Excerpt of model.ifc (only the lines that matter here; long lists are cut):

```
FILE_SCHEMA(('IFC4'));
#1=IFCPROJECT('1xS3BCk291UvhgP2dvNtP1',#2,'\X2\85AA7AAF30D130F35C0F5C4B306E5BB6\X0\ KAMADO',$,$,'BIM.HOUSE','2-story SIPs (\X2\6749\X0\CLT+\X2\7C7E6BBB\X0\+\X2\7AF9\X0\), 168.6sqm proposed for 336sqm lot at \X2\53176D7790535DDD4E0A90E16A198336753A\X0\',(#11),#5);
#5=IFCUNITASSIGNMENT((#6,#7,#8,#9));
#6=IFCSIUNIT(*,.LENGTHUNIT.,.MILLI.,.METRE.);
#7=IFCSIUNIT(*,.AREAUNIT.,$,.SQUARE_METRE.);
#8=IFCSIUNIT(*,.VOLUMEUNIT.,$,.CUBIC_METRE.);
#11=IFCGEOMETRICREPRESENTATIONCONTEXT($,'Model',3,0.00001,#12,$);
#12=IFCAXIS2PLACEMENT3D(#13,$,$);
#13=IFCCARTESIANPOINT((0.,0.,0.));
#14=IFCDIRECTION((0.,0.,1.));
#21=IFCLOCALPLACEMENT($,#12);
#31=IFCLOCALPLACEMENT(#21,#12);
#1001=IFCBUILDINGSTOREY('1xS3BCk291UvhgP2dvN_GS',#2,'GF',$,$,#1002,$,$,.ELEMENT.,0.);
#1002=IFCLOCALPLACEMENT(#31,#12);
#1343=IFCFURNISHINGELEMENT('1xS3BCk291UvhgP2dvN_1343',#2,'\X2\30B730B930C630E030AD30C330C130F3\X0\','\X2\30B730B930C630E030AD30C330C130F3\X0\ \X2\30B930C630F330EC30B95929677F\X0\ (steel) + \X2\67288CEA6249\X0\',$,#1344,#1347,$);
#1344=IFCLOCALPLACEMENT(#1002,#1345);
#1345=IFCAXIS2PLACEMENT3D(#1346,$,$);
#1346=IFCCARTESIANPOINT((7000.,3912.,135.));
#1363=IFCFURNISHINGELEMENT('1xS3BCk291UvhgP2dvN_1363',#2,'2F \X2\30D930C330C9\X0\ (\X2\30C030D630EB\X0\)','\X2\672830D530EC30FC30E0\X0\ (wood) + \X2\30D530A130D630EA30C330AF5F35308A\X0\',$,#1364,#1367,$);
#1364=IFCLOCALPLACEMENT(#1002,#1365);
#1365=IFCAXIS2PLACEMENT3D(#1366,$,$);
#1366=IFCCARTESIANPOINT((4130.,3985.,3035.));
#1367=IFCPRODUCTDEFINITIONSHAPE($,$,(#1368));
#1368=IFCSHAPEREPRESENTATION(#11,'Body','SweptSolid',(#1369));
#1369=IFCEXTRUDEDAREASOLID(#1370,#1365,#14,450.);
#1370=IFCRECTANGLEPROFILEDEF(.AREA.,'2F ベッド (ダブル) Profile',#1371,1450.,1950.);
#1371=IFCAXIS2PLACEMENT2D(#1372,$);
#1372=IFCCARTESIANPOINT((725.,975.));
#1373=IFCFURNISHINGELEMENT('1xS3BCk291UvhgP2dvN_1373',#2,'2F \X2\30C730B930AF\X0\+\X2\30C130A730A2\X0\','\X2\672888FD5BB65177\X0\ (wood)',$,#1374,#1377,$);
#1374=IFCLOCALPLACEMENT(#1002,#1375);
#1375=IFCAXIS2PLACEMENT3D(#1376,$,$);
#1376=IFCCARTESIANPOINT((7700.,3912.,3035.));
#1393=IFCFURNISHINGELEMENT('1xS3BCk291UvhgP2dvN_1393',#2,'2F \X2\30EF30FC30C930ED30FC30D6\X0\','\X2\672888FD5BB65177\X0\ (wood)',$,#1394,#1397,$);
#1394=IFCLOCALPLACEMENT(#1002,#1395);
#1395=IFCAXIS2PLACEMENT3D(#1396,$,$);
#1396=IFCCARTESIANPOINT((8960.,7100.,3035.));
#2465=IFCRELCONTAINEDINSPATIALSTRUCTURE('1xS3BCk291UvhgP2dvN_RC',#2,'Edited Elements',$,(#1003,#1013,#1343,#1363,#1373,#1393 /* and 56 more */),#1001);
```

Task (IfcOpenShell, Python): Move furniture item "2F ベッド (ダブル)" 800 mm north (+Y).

```python
import ifcopenshell
import ifcopenshell.api.geometry
import ifcopenshell.util.placement
import ifcopenshell.util.unit

model = ifcopenshell.open("model.ifc")
unit_scale = ifcopenshell.util.unit.calculate_unit_scale(model)

item = model.by_id(1363)
matrix = ifcopenshell.util.placement.get_local_placement(item.ObjectPlacement)
matrix[1, 3] += 0.8 / unit_scale
ifcopenshell.api.geometry.edit_object_placement(model, product=item, matrix=matrix, is_si=False)

print(ifcopenshell.util.placement.get_local_placement(item.ObjectPlacement).round(3) + 0.0)

model.write("model_rev.ifc")
```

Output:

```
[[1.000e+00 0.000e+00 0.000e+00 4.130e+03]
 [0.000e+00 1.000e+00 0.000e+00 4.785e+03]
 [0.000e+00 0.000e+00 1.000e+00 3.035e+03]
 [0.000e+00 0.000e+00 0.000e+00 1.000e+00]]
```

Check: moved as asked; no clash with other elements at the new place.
